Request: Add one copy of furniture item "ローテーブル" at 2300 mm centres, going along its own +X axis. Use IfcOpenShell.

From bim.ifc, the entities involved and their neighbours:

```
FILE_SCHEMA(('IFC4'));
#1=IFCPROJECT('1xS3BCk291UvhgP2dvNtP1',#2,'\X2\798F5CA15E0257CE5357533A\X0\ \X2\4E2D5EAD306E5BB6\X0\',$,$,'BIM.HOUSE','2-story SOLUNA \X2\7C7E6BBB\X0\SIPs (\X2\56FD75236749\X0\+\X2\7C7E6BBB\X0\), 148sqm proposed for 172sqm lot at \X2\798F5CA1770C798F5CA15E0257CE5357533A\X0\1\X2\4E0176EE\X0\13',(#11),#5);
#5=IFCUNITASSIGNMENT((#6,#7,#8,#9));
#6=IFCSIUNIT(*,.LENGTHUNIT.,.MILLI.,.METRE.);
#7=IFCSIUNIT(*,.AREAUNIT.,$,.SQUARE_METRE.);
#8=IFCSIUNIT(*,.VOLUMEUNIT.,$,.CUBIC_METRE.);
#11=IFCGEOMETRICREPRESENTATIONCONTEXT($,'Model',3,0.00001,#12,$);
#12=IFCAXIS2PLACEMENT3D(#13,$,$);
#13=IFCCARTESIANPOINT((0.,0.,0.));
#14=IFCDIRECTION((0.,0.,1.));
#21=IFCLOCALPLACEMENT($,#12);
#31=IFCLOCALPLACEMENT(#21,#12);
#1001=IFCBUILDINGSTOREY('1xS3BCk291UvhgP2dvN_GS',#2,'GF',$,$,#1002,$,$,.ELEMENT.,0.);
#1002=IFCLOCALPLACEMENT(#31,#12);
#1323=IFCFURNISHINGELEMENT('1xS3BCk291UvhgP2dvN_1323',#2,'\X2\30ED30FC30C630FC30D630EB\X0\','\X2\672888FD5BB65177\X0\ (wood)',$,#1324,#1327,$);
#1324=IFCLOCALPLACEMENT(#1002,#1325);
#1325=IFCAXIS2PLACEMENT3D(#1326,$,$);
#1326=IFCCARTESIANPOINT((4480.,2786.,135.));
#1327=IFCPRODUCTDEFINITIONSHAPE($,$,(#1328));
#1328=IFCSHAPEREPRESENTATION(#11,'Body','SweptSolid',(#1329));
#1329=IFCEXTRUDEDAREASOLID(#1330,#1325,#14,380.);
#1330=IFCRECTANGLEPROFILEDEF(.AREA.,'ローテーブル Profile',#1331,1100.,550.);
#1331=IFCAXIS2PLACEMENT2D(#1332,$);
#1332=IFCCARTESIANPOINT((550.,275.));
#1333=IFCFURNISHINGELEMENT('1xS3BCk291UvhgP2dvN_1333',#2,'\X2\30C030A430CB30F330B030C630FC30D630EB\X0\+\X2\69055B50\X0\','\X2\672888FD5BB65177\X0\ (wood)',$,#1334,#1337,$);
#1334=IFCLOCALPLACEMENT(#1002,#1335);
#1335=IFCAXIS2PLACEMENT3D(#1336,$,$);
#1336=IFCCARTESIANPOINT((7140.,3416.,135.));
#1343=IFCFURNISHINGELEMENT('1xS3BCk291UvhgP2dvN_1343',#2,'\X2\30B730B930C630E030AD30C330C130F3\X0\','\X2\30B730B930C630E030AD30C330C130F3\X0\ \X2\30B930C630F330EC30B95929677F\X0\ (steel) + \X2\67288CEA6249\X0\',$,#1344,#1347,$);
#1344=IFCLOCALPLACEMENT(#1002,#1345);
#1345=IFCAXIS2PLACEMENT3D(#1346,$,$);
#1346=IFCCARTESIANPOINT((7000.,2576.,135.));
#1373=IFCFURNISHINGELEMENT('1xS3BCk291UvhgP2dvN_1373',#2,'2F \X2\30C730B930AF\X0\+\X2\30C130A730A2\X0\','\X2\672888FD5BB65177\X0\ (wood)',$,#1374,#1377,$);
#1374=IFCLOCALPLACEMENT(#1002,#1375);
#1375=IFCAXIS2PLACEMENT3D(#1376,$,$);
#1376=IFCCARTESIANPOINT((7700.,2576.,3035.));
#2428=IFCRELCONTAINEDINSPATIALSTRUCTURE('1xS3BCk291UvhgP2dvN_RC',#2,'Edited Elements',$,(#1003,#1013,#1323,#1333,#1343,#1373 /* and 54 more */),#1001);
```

```python
import ifcopenshell
import ifcopenshell.api.geometry
import ifcopenshell.api.root
import ifcopenshell.util.element
import ifcopenshell.util.placement
import ifcopenshell.util.unit

model = ifcopenshell.open("bim.ifc")
unit_scale = ifcopenshell.util.unit.calculate_unit_scale(model)


def reuse_history(source, copy):
    """copy_class also copies each property set's owner history, people and application; keep the originals."""
    for rel in copy.IsDefinedBy:
        if rel.is_a("IfcRelDefinesByProperties") and (history := rel.RelatingPropertyDefinition.OwnerHistory):
            rel.RelatingPropertyDefinition.OwnerHistory = source.OwnerHistory
            ifcopenshell.util.element.remove_deep2(model, history)


source = model.by_guid("1xS3BCk291UvhgP2dvN_1323")
base = ifcopenshell.util.placement.get_local_placement(source.ObjectPlacement)
step = base[:3, 0] * 2.3 / unit_scale

for i in range(1, 2):
    copy = ifcopenshell.api.root.copy_class(model, product=source)
    copy.Representation = ifcopenshell.util.element.copy_deep(
        model, source.Representation, exclude=["IfcGeometricRepresentationContext", "IfcRepresentationMap"]
    )
    reuse_history(source, copy)
    matrix = base.copy()
    matrix[:3, 3] += i * step
    print("added at", matrix[:3, 3].round(3) + 0.0)
    ifcopenshell.api.geometry.edit_object_placement(model, product=copy, matrix=matrix, is_si=False)

model.write("bim_edited.ifc")
```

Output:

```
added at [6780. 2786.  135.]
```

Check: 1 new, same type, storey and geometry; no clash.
